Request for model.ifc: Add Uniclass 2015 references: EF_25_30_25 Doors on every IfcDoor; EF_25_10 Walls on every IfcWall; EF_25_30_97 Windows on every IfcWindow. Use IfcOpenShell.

First a look at what the model holds.

```python
import ifcopenshell

model = ifcopenshell.open("model.ifc")
print(model.schema)
print("classifications:", [c.Name for c in model.by_type("IfcClassification")])
for ifc_class in ("IfcDoor", "IfcRoof", "IfcStair", "IfcWall", "IfcWindow"):
    print(ifc_class, len(model.by_type(ifc_class)))
```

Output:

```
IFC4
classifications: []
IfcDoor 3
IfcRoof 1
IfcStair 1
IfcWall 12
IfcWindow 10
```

```python
import ifcopenshell
import ifcopenshell.api.classification

model = ifcopenshell.open("model.ifc")

system = ifcopenshell.api.classification.add_classification(model, classification="Uniclass 2015")

codes = {
    "IfcDoor": ("EF_25_30_25", "Doors"),
    "IfcWall": ("EF_25_10", "Walls"),
    "IfcWindow": ("EF_25_30_97", "Windows"),
}
for ifc_class, (code, name) in codes.items():
    products = model.by_type(ifc_class)
    ifcopenshell.api.classification.add_reference(
        model, products=products, classification=system, identification=code, name=name
    )
    print(code, len(products))

model.write("model-out.ifc")
```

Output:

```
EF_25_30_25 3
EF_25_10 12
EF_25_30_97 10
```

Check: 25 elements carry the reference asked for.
